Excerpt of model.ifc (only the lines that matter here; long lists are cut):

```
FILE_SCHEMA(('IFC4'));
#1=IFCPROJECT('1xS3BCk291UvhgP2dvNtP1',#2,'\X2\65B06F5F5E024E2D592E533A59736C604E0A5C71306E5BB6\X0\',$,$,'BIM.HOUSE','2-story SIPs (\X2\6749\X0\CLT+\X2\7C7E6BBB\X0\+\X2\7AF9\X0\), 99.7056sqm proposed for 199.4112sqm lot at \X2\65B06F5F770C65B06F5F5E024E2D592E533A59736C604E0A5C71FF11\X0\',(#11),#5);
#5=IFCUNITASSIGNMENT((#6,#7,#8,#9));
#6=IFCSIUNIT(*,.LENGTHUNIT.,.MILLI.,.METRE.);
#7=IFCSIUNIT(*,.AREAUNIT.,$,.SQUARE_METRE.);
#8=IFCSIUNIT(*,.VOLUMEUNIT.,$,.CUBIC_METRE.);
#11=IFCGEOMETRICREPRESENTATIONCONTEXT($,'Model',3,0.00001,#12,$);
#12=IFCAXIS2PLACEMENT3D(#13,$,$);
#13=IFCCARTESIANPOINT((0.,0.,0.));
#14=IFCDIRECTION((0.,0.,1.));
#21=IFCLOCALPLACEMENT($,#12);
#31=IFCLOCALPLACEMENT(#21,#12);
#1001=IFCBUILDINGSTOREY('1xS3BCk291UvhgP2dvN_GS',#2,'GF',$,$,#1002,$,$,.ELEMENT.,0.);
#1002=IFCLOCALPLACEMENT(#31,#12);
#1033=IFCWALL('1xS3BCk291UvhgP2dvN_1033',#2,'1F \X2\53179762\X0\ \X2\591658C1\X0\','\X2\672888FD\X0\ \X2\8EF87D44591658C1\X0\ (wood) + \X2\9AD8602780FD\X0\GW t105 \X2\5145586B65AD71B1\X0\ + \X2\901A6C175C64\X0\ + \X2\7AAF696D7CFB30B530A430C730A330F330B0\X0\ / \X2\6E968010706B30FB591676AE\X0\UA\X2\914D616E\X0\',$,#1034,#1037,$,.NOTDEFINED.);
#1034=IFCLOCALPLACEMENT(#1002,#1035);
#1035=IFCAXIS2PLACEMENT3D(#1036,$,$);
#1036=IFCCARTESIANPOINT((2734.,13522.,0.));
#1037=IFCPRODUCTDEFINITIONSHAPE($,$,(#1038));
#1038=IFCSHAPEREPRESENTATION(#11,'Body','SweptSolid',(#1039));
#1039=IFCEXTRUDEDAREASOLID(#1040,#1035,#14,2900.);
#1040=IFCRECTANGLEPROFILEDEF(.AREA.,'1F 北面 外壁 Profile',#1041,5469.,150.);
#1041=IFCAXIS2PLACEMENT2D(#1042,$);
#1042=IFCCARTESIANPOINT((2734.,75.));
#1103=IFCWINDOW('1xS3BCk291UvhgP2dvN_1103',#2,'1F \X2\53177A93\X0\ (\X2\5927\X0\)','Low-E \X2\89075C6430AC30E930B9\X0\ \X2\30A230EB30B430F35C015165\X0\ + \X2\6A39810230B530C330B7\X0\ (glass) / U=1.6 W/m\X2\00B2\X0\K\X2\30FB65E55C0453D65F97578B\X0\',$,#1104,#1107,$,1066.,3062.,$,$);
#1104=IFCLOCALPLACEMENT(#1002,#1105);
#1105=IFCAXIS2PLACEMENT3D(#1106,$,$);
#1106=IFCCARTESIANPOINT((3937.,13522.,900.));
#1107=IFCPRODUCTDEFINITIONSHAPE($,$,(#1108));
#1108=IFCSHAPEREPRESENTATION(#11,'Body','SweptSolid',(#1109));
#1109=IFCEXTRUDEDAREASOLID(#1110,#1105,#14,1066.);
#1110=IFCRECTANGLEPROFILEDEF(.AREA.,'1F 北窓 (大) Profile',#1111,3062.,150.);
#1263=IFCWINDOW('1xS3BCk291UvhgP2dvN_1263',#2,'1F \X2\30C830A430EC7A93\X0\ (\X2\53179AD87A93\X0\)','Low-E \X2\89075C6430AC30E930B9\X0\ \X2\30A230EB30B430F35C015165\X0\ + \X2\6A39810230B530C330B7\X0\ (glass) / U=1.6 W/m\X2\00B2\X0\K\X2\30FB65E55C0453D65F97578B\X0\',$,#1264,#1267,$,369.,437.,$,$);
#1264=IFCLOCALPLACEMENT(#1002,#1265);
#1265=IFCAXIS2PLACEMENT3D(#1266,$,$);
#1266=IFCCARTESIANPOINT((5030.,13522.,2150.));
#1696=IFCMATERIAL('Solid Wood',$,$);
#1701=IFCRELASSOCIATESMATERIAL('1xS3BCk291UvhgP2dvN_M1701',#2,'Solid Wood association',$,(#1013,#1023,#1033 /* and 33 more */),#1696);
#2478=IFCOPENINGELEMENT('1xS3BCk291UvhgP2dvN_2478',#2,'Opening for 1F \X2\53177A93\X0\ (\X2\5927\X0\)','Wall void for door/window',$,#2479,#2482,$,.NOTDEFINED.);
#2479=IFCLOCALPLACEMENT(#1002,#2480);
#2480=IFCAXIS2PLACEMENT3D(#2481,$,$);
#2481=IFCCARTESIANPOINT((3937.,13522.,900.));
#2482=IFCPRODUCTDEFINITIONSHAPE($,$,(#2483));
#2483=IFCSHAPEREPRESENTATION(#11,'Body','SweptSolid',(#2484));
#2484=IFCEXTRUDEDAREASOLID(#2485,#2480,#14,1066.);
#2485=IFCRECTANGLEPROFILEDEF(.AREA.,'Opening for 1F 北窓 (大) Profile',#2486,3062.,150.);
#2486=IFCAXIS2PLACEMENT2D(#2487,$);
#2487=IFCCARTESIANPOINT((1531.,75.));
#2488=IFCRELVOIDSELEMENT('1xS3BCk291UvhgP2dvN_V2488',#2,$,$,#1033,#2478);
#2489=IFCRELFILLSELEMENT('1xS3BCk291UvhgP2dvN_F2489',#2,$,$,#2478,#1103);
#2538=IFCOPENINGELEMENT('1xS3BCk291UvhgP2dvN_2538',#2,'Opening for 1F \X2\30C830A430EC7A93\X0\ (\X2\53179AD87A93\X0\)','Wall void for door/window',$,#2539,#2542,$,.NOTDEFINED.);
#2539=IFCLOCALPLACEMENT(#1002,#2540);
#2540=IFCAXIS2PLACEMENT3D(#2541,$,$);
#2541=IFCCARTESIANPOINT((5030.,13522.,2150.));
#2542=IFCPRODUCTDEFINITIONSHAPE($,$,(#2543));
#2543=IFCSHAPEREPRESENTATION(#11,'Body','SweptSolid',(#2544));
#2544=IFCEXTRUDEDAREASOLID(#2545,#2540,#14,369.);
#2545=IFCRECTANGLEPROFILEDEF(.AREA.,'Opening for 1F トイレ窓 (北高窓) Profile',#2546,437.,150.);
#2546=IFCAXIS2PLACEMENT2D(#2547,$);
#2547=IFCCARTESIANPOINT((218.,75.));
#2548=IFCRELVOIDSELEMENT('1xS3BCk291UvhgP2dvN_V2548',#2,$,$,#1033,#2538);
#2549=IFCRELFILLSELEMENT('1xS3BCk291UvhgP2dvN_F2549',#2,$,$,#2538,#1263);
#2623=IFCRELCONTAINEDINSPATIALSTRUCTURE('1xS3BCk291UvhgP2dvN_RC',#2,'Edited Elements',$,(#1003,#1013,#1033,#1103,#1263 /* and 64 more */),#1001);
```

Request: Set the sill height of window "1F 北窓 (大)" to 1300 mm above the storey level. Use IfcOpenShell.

```python
import numpy as np
import ifcopenshell
import ifcopenshell.api.geometry
import ifcopenshell.geom
import ifcopenshell.util.element
import ifcopenshell.util.placement
import ifcopenshell.util.shape
import ifcopenshell.util.unit

model = ifcopenshell.open("model.ifc")
unit_scale = ifcopenshell.util.unit.calculate_unit_scale(model)

window = model.by_guid("1xS3BCk291UvhgP2dvN_1103")
opening = window.FillsVoids[0].RelatingOpeningElement
storey = ifcopenshell.util.element.get_container(window, ifc_class="IfcBuildingStorey")
level = ifcopenshell.util.placement.get_local_placement(storey.ObjectPlacement)[2, 3]

# The opening's origin need not be at the sill, so measure its lowest point.
shape = ifcopenshell.geom.create_shape(ifcopenshell.geom.settings(), opening)
bottom = ifcopenshell.util.shape.get_shape_bottom_elevation(shape, shape.geometry) / unit_scale
dz = level + 1300.0 - bottom

shift = np.array([0.0, 0.0, dz])
# The window is not placed relative to its opening, so move both.
for product in (opening, window):
    matrix = ifcopenshell.util.placement.get_local_placement(product.ObjectPlacement)
    matrix[:3, 3] += shift
    ifcopenshell.api.geometry.edit_object_placement(model, product=product, matrix=matrix, is_si=False)

print(f"moved by {dz * unit_scale:+.3f} m")

model.write("model_updated.ifc")
```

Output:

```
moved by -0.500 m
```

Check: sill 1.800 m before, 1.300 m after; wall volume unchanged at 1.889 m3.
